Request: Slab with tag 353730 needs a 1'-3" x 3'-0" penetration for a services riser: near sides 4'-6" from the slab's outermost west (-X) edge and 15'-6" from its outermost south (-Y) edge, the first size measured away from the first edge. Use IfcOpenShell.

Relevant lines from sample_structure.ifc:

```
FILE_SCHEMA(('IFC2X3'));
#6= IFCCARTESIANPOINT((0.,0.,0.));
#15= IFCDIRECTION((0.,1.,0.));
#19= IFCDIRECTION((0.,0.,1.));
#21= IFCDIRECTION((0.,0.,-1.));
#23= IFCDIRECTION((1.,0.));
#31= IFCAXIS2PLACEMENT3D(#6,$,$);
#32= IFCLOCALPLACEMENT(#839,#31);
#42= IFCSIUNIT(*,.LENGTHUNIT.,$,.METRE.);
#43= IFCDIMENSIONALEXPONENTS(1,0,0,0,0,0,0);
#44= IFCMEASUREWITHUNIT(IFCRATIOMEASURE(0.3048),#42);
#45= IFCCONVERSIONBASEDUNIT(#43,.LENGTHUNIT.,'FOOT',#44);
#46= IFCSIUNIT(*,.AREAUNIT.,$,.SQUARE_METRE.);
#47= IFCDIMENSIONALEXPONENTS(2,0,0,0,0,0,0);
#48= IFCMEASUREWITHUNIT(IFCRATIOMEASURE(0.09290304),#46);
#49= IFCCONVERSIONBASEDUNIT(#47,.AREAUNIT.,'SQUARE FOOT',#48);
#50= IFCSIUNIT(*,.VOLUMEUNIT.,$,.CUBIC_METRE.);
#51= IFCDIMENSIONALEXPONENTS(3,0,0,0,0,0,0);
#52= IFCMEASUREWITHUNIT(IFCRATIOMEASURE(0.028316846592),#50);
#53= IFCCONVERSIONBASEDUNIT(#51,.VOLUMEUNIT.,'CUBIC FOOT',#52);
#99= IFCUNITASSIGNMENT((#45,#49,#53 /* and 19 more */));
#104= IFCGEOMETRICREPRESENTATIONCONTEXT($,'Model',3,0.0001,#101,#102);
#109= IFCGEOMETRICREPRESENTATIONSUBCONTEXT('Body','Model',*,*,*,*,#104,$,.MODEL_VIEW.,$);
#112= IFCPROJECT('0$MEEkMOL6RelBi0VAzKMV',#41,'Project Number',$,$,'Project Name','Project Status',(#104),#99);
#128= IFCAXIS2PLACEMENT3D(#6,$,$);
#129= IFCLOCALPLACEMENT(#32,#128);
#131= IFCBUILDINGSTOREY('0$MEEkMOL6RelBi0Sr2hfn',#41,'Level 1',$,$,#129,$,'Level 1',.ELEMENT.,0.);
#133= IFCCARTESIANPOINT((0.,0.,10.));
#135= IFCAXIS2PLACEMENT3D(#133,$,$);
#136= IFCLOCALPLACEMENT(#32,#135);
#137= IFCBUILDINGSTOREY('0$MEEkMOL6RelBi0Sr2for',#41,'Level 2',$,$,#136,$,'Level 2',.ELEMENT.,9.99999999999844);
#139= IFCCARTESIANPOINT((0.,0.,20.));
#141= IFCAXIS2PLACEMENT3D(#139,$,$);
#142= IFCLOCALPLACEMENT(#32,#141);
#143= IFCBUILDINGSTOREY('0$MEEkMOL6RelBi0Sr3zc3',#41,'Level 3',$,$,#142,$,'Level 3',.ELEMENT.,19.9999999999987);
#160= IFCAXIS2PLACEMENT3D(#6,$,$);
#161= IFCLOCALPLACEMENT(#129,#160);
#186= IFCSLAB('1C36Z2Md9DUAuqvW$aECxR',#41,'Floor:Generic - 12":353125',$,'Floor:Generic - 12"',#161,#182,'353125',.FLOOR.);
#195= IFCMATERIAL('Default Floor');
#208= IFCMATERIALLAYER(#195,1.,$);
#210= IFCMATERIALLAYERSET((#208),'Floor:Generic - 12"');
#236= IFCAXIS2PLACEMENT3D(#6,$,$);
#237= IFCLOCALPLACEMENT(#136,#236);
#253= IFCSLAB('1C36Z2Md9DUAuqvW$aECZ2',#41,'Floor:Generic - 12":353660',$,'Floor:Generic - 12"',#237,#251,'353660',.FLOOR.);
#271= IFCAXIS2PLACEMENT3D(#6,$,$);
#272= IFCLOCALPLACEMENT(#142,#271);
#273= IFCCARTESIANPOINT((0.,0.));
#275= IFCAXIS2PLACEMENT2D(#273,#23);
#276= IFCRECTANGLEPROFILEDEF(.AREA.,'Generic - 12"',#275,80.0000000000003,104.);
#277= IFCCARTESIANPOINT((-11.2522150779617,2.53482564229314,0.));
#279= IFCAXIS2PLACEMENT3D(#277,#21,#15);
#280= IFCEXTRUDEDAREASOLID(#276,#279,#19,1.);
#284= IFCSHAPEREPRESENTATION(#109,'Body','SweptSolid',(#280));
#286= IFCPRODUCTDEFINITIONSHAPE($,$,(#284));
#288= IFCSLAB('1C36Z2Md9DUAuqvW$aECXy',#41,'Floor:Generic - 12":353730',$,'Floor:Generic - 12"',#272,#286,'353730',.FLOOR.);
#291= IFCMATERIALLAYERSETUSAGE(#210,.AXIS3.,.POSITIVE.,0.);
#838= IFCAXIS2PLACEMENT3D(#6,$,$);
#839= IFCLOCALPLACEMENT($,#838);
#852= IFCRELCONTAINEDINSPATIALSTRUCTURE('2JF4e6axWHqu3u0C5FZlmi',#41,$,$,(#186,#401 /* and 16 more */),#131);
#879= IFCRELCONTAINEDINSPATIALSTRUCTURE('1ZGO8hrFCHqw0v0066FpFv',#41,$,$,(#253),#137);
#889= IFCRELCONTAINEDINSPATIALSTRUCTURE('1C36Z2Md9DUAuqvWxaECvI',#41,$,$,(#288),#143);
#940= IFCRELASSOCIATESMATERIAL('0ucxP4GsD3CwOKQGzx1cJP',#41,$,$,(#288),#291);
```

```python
import numpy as np
import ifcopenshell
import ifcopenshell.api.feature
import ifcopenshell.api.geometry
import ifcopenshell.api.root
import ifcopenshell.geom
import ifcopenshell.util.placement
import ifcopenshell.util.representation
import ifcopenshell.util.shape
import ifcopenshell.util.unit

model = ifcopenshell.open("sample_structure.ifc")
unit_scale = ifcopenshell.util.unit.calculate_unit_scale(model)
settings = ifcopenshell.geom.settings()


def volume(element):
    """Net volume in cubic metres, openings subtracted."""
    shape = ifcopenshell.geom.create_shape(settings, element)
    return ifcopenshell.util.shape.get_volume(shape.geometry)


slab = model.by_id(288)
before = volume(slab)

# Extent in the slab's own axes, in metres. The edges named are its -X and -Y sides.
slab_shape = ifcopenshell.geom.create_shape(settings, slab)
vertices = ifcopenshell.util.shape.get_vertices(slab_shape.geometry)
x_min, y_min, bottom = vertices.min(axis=0)
top = vertices[:, 2].max()

opening = ifcopenshell.api.root.create_entity(model, ifc_class="IfcOpeningElement", name="Services riser opening")
context = ifcopenshell.util.representation.get_context(model, "Model", "Body", "MODEL_VIEW")
width, depth = 0.381, 0.9144
outline = [(0.0, 0.0), (width, 0.0), (width, depth), (0.0, depth), (0.0, 0.0)]
# Overshoot both faces by 50 mm so the cut is clean.
shape = ifcopenshell.api.geometry.add_slab_representation(
    model, context=context, depth=top - bottom + 0.1, polyline=outline
)
ifcopenshell.api.geometry.assign_representation(model, product=opening, representation=shape)

matrix = ifcopenshell.util.placement.get_local_placement(slab.ObjectPlacement)
matrix[:, 3] = matrix @ np.append(np.array([x_min + 1.3716, y_min + 4.7244, bottom - 0.05]) / unit_scale, 1.0)
ifcopenshell.api.geometry.edit_object_placement(model, product=opening, matrix=matrix, is_si=False)
ifcopenshell.api.feature.add_feature(model, feature=opening, element=slab)

after = volume(slab)

print(f"slab volume {before:.3f} -> {after:.3f} m3")

model.write("sample_structure_updated.ifc")
```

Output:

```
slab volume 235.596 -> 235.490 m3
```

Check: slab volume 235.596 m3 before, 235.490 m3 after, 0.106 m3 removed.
